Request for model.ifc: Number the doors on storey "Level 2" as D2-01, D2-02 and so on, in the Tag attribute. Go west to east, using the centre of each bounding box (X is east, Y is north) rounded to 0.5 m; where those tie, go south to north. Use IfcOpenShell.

First a look at what the model holds.

```python
import ifcopenshell
import ifcopenshell.util.element
import ifcopenshell.util.placement

model = ifcopenshell.open("model.ifc")
print(model.schema)
storey = next(s for s in model.by_type("IfcBuildingStorey") if s.Name == "Level 2")
doors = [e for e in ifcopenshell.util.element.get_decomposition(storey) if e.is_a("IfcDoor")]
for e in sorted(doors, key=lambda e: e.id()):
    origin = ifcopenshell.util.placement.get_local_placement(e.ObjectPlacement)[:3, 3]
    print(e.id(), e.Tag, e.Name, origin.round(2) + 0.0, sep=" | ")
```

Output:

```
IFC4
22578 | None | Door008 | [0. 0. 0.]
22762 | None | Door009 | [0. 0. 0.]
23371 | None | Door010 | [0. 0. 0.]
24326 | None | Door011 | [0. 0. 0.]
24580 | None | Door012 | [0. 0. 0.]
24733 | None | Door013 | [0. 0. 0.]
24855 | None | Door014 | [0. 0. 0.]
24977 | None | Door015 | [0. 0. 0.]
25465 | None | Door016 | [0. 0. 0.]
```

```python
import ifcopenshell
import ifcopenshell.geom
import ifcopenshell.util.element
import ifcopenshell.util.shape

model = ifcopenshell.open("model.ifc")
settings = ifcopenshell.geom.settings()
settings.set("use-world-coords", True)


def centre(element):
    shape = ifcopenshell.geom.create_shape(settings, element)
    return ifcopenshell.util.shape.get_bbox_centroid(shape.geometry)


storey = next(s for s in model.by_type("IfcBuildingStorey") if s.Name == "Level 2")
doors = [e for e in ifcopenshell.util.element.get_decomposition(storey) if e.is_a("IfcDoor")]

# Insertion points can sit at a corner or the storey origin, so sort by the geometry (in metres).
centres = {e: centre(e) for e in doors}
doors.sort(key=lambda e: (round(centres[e][0] / 0.5), centres[e][1]))

for i, e in enumerate(doors, start=1):
    number = f"D2-{i:02d}"
    e.Tag = number
    print(e.id(), number)

model.write("model_updated.ifc")
```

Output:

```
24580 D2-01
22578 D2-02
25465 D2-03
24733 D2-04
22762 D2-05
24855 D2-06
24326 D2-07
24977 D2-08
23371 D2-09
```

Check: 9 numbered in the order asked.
